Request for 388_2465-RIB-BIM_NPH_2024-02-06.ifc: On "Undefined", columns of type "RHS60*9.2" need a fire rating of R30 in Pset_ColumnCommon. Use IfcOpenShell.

First a look at what the model holds.

```python
import ifcopenshell
import ifcopenshell.util.element

model = ifcopenshell.open("388_2465-RIB-BIM_NPH_2024-02-06.ifc")
print(model.schema)
storey = next(s for s in model.by_type("IfcBuildingStorey") if s.Name == "Undefined")
columns = [e for e in ifcopenshell.util.element.get_decomposition(storey) if e.is_a("IfcColumn")]
seen = {}
for e in columns:
    element_type = ifcopenshell.util.element.get_type(e)
    key = (element_type.Name if element_type != e and element_type else None, ifcopenshell.util.element.get_pset(e, "Pset_ColumnCommon", "FireRating"))
    seen[key] = seen.get(key, 0) + 1
for (name, value), count in sorted(seen.items(), key=str):
    print(count, "x", name, "|", value)
```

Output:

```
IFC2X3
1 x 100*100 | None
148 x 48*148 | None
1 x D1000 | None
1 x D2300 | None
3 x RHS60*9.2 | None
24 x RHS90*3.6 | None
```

```python
import ifcopenshell
import ifcopenshell.api.pset
import ifcopenshell.util.element

model = ifcopenshell.open("388_2465-RIB-BIM_NPH_2024-02-06.ifc")

storey = next(s for s in model.by_type("IfcBuildingStorey") if s.Name == "Undefined")
columns = [e for e in ifcopenshell.util.element.get_decomposition(storey) if e.is_a("IfcColumn")]

count = 0
for e in columns:
    element_type = ifcopenshell.util.element.get_type(e)
    if element_type in (None, e) or element_type.Name != "RHS60*9.2":
        continue
    found = ifcopenshell.util.element.get_pset(e, "Pset_ColumnCommon", should_inherit=False)
    if found:
        pset = model.by_id(found["id"])
        if len(ifcopenshell.util.element.get_elements_by_pset(pset)) > 1:
            pset = ifcopenshell.api.pset.unshare_pset(model, products=[e], pset=pset)[0]
    else:
        pset = ifcopenshell.api.pset.add_pset(model, product=e, name="Pset_ColumnCommon")
    ifcopenshell.api.pset.edit_pset(model, pset=pset, properties={"FireRating": "R30"})
    count += 1

print(count, "columns updated")

model.write("388_2465-RIB-BIM_NPH_2024-02-06_updated.ifc")
```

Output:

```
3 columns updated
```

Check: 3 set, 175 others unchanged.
